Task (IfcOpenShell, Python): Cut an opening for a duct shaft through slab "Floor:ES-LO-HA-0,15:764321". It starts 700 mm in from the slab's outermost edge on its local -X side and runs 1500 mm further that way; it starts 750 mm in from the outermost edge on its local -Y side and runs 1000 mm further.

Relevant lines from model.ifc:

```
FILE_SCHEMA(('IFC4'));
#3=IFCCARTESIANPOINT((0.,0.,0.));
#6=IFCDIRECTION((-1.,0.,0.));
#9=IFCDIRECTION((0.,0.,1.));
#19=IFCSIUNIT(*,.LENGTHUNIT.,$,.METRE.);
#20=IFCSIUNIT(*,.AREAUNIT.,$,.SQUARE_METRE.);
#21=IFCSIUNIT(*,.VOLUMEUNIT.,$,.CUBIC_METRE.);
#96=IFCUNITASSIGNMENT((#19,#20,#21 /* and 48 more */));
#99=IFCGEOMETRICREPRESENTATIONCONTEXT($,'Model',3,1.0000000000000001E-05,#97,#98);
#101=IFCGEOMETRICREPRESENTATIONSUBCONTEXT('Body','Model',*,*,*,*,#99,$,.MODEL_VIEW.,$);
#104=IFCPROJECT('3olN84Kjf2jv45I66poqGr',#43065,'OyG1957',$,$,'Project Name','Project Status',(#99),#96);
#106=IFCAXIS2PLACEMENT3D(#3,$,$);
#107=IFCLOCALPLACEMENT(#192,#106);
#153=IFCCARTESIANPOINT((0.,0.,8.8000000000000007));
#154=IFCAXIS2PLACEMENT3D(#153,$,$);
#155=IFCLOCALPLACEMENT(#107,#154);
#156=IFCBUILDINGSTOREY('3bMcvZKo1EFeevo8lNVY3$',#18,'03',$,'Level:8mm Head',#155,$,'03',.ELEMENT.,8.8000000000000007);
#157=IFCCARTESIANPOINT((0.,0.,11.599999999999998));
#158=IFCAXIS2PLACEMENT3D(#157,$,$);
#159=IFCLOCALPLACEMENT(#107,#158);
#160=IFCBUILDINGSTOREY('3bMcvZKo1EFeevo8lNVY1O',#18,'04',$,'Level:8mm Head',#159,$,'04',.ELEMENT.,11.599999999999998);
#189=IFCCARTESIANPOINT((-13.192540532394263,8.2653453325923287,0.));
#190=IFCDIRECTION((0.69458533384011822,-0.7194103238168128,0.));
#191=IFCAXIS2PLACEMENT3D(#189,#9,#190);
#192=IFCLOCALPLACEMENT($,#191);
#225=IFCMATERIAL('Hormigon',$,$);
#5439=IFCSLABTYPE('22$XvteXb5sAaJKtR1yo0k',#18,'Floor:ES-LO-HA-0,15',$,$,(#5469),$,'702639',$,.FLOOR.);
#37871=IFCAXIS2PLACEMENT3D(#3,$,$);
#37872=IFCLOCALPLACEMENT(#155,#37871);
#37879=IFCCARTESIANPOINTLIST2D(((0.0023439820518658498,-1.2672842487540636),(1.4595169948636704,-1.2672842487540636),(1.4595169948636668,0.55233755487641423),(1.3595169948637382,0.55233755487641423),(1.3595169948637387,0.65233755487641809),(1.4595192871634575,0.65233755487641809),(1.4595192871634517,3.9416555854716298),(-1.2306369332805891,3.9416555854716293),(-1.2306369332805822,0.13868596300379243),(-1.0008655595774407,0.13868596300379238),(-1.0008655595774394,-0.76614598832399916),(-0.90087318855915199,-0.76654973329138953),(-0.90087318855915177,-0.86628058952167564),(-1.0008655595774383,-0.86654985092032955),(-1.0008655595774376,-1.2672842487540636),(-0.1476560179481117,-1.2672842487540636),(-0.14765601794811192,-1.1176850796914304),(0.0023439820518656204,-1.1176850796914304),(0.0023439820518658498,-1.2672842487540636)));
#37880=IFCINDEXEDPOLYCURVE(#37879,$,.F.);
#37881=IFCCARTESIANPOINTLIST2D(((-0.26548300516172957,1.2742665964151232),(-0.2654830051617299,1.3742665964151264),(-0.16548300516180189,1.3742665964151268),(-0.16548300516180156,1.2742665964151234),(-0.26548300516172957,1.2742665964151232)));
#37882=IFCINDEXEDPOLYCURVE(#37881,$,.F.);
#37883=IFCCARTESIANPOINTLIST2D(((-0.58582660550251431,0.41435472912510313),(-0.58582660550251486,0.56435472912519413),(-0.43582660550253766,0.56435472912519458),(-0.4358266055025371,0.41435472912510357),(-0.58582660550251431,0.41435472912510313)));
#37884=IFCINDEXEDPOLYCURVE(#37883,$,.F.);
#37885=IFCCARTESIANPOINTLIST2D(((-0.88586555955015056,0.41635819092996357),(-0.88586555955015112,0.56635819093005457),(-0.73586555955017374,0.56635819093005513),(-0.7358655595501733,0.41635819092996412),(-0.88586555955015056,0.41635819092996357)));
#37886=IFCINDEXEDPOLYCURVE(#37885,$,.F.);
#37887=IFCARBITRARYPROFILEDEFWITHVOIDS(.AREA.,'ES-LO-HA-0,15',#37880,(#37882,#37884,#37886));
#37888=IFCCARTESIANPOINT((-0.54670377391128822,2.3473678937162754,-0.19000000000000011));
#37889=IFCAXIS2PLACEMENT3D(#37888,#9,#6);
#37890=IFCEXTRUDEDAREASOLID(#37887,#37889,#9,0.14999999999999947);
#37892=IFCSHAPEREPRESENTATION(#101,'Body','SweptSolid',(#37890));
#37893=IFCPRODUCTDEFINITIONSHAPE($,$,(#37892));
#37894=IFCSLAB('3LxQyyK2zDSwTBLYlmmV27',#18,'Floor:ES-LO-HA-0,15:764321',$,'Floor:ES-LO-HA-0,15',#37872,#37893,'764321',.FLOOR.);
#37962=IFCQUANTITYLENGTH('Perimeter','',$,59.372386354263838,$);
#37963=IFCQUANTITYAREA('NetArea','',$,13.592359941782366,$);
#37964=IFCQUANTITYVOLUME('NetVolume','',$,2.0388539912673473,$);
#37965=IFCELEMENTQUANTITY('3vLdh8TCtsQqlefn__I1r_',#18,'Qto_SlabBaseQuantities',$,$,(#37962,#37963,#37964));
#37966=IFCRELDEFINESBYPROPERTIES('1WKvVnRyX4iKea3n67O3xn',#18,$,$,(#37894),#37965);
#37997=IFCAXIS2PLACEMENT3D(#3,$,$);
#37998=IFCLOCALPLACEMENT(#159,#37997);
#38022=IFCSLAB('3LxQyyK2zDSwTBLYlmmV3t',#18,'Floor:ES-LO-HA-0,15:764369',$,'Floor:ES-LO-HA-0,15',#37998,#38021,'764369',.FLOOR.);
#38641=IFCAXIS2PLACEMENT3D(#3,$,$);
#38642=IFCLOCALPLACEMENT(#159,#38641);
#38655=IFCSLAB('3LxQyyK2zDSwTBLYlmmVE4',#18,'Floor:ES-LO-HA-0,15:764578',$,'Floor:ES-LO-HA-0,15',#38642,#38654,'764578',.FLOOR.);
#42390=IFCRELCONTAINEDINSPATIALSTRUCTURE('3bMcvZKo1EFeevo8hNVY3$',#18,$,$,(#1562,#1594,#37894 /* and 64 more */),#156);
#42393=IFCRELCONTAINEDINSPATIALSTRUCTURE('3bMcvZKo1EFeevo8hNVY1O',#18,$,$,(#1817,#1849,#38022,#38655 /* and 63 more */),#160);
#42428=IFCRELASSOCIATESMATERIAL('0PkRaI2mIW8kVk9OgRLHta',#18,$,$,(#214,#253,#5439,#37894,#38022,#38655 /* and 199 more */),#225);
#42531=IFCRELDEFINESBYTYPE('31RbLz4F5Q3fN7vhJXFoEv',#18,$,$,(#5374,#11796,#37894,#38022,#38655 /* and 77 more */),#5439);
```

```python
import numpy as np
import ifcopenshell
import ifcopenshell.api.feature
import ifcopenshell.api.geometry
import ifcopenshell.api.pset
import ifcopenshell.api.root
import ifcopenshell.geom
import ifcopenshell.util.element
import ifcopenshell.util.placement
import ifcopenshell.util.representation
import ifcopenshell.util.shape
import ifcopenshell.util.unit

model = ifcopenshell.open("model.ifc")
unit_scale = ifcopenshell.util.unit.calculate_unit_scale(model)
area_scale = ifcopenshell.util.unit.calculate_unit_scale(model, "AREAUNIT")
volume_scale = ifcopenshell.util.unit.calculate_unit_scale(model, "VOLUMEUNIT")
settings = ifcopenshell.geom.settings()


def volume(element):
    """Net volume in cubic metres, openings subtracted."""
    shape = ifcopenshell.geom.create_shape(settings, element)
    return ifcopenshell.util.shape.get_volume(shape.geometry)


slab = model.by_id(37894)
before = volume(slab)

# Extent in the slab's own axes, in metres. The edges named are its -X and -Y sides.
slab_shape = ifcopenshell.geom.create_shape(settings, slab)
vertices = ifcopenshell.util.shape.get_vertices(slab_shape.geometry)
x_min, y_min, bottom = vertices.min(axis=0)
top = vertices[:, 2].max()

opening = ifcopenshell.api.root.create_entity(model, ifc_class="IfcOpeningElement", name="Duct shaft opening", predefined_type="OPENING")
context = ifcopenshell.util.representation.get_context(model, "Model", "Body", "MODEL_VIEW")
width, depth = 1.5, 1
outline = [(0.0, 0.0), (width, 0.0), (width, depth), (0.0, depth), (0.0, 0.0)]
# Overshoot both faces by 50 mm so the cut is clean.
shape = ifcopenshell.api.geometry.add_slab_representation(
    model, context=context, depth=top - bottom + 0.1, polyline=outline
)
ifcopenshell.api.geometry.assign_representation(model, product=opening, representation=shape)

matrix = ifcopenshell.util.placement.get_local_placement(slab.ObjectPlacement)
matrix[:, 3] = matrix @ np.append(np.array([x_min + 0.7, y_min + 0.75, bottom - 0.05]) / unit_scale, 1.0)
ifcopenshell.api.geometry.edit_object_placement(model, product=opening, matrix=matrix, is_si=False)
ifcopenshell.api.feature.add_feature(model, feature=opening, element=slab)

after = volume(slab)

# Update the slab's stored quantities.
qto = model.by_id(ifcopenshell.util.element.get_pset(slab, "Qto_SlabBaseQuantities", should_inherit=False)["id"])
ifcopenshell.api.pset.edit_qto(model, qto=qto, properties={
    "NetArea": after / (top - bottom) / area_scale,
    "NetVolume": after / volume_scale,
})

print(f"slab volume {before:.3f} -> {after:.3f} m3")

model.write("model-out.ifc")
```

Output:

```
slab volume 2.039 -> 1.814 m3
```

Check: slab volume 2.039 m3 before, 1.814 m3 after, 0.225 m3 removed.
